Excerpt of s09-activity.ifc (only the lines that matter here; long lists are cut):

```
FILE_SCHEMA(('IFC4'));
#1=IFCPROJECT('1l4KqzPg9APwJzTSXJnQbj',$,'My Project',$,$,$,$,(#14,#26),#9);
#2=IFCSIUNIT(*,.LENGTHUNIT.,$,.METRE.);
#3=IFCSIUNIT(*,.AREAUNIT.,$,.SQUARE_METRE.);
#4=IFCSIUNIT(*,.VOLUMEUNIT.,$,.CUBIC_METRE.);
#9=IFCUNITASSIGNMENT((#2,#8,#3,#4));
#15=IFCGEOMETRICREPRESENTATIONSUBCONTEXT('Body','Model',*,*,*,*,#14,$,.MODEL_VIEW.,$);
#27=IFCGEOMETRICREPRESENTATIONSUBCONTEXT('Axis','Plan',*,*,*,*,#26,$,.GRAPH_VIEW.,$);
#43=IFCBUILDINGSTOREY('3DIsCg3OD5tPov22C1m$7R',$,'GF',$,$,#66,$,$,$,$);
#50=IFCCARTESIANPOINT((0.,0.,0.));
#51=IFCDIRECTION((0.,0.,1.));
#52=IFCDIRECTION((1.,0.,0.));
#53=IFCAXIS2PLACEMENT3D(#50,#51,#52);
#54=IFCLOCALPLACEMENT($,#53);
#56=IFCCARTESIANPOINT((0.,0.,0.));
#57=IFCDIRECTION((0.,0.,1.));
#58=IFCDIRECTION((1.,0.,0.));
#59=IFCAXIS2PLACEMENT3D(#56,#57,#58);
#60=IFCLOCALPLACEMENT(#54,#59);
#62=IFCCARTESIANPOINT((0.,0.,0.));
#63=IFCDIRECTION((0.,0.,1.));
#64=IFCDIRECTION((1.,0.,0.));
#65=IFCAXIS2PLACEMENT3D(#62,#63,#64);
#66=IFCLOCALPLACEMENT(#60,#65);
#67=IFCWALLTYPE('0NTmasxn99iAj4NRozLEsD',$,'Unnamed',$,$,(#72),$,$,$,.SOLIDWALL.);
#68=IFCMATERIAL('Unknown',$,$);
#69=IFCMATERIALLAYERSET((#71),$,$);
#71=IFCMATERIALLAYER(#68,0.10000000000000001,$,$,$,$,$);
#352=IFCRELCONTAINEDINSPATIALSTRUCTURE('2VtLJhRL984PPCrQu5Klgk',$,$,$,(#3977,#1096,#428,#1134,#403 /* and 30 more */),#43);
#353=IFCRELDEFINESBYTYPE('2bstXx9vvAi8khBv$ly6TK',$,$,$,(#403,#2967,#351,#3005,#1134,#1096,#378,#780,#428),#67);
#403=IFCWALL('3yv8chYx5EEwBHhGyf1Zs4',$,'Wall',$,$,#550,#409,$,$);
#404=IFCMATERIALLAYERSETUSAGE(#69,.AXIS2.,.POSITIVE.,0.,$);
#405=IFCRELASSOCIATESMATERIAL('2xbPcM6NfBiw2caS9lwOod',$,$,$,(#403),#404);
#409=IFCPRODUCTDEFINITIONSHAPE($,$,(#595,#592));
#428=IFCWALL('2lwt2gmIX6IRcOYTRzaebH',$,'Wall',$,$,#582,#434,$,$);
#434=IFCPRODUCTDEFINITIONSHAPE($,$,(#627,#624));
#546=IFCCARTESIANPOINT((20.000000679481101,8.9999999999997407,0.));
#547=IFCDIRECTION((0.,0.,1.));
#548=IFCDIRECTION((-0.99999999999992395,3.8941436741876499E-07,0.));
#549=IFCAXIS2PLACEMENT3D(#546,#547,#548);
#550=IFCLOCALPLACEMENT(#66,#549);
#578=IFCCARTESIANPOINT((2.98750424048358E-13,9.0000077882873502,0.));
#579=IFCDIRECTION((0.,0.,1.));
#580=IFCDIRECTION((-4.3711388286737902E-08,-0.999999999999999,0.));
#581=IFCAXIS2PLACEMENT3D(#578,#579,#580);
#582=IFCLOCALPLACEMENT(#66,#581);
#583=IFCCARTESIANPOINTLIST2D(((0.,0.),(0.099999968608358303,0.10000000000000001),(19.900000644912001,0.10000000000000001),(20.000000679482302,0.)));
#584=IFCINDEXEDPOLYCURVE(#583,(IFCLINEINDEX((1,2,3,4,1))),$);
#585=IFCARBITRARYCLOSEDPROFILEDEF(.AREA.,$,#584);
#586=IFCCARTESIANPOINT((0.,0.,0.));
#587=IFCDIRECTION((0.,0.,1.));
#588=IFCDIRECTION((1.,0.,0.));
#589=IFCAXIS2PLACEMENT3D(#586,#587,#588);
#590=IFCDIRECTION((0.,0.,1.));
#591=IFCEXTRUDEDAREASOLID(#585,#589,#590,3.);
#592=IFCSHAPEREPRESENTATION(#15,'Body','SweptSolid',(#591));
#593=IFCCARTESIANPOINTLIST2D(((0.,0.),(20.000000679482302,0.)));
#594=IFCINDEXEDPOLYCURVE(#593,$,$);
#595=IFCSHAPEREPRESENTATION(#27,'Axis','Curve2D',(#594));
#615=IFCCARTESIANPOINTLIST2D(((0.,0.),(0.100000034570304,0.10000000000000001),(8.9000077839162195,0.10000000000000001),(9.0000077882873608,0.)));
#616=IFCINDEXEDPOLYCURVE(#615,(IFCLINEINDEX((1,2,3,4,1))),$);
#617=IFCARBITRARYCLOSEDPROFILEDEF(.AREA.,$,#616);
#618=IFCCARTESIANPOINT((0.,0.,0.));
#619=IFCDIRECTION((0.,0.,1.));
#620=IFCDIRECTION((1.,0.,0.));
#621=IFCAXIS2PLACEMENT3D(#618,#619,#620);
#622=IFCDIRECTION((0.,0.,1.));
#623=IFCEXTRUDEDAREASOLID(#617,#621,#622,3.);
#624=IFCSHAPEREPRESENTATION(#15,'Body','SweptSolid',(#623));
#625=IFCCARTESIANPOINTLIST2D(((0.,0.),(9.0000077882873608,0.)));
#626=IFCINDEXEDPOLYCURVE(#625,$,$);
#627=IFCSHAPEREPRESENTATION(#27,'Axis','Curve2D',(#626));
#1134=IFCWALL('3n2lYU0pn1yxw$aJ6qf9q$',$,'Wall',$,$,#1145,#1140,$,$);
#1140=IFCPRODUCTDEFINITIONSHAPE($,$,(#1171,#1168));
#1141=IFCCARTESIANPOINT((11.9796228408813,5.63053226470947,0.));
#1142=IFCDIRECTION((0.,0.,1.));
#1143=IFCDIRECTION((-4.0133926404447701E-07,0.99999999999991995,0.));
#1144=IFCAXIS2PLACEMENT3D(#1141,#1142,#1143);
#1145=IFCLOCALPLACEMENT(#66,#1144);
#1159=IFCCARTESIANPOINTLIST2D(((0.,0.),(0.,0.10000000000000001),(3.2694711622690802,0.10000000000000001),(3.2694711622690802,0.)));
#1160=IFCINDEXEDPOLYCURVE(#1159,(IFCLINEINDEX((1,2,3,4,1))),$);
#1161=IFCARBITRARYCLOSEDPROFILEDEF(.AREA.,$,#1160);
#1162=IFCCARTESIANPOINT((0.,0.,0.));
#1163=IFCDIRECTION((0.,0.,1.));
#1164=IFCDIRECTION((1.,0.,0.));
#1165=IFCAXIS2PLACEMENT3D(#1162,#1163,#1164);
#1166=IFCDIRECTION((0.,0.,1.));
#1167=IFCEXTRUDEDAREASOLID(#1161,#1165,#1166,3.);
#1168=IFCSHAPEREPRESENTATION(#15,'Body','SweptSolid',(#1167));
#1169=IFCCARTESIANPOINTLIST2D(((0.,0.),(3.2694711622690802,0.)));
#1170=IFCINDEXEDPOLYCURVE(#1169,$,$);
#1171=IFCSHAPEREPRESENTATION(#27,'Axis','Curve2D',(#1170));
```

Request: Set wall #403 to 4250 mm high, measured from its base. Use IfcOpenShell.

```python
import ifcopenshell
import ifcopenshell.geom
import ifcopenshell.util.representation
import ifcopenshell.util.shape
import ifcopenshell.util.unit

model = ifcopenshell.open("s09-activity.ifc")
unit_scale = ifcopenshell.util.unit.calculate_unit_scale(model)
settings = ifcopenshell.geom.settings()


def volume(element):
    """Net volume in cubic metres, openings subtracted."""
    shape = ifcopenshell.geom.create_shape(settings, element)
    return ifcopenshell.util.shape.get_volume(shape.geometry)


wall = model.by_id(403)
before = volume(wall)

body = ifcopenshell.util.representation.get_representation(wall, "Model", "Body")
solid = body.Items[0]
old_height = solid.Depth
solid.Depth = 4.25 / unit_scale
after = volume(wall)

print(f"height {old_height:g} -> {solid.Depth:g}, volume {before:.3f} -> {after:.3f} m3")

model.write("s09-activity_edited.ifc")
```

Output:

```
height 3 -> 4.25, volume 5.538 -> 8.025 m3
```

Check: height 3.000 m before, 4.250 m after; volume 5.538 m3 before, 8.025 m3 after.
